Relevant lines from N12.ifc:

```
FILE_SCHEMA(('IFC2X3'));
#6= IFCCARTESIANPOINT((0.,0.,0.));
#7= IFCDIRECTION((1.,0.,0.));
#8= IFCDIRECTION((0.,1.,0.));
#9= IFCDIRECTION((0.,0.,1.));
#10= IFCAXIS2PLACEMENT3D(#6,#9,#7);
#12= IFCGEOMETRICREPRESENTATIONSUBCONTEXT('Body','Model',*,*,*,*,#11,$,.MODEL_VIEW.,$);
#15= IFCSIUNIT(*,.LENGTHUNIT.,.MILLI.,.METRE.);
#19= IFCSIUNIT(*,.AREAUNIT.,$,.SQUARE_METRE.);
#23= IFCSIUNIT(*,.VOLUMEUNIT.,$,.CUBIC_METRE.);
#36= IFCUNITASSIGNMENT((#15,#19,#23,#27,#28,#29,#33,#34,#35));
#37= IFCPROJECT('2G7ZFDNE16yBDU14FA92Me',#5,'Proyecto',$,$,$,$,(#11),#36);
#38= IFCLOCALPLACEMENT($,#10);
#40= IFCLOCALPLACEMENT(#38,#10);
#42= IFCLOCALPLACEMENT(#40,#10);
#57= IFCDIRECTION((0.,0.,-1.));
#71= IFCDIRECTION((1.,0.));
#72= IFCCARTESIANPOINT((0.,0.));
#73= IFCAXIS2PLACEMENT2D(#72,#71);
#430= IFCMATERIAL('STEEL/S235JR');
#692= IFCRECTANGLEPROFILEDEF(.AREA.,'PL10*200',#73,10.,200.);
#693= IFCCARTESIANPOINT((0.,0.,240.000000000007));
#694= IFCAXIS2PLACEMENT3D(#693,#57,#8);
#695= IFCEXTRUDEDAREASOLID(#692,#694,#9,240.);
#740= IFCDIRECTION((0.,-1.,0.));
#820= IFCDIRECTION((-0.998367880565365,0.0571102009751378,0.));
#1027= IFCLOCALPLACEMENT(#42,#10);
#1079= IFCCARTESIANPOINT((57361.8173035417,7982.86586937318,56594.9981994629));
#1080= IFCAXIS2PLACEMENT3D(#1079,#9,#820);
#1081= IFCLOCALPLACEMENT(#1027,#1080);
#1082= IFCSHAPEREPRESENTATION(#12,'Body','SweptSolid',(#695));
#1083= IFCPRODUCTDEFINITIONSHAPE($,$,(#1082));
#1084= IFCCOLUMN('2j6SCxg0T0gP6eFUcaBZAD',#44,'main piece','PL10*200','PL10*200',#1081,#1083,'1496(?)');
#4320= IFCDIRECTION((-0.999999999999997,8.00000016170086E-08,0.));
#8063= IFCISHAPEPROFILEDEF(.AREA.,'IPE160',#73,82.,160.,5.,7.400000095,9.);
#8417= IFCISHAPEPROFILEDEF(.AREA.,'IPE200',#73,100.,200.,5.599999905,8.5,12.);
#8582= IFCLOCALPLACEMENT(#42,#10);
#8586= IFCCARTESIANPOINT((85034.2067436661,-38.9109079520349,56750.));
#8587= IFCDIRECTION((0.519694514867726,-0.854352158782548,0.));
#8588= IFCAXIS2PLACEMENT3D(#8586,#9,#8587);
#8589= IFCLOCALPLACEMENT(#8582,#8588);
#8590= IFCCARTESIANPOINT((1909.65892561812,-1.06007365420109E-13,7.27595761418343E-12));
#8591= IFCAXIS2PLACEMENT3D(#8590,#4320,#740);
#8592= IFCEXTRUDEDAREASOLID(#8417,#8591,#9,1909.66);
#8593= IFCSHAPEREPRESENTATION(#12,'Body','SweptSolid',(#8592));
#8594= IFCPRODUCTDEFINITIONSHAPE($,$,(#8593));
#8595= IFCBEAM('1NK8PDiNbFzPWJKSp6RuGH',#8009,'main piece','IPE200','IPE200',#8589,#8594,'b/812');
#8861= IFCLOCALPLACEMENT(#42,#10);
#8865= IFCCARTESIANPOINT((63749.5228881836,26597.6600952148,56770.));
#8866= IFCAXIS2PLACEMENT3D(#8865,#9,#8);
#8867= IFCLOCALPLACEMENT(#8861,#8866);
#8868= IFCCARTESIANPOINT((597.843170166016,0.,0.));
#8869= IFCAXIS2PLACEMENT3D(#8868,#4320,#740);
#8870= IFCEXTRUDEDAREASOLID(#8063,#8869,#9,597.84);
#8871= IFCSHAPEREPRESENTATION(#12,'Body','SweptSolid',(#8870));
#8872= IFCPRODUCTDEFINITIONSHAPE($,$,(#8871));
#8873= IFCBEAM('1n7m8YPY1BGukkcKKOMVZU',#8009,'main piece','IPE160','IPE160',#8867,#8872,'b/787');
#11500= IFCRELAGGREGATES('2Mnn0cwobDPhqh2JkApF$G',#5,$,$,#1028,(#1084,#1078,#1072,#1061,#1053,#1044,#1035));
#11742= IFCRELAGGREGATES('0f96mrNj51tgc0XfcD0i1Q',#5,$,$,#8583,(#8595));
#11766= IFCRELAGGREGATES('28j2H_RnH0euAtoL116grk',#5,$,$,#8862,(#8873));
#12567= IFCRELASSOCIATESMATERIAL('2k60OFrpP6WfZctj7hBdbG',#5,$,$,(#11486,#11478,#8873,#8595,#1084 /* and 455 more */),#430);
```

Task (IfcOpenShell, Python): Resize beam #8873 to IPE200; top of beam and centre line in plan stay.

```python
import ifcopenshell
import ifcopenshell.util.element
import ifcopenshell.util.representation

model = ifcopenshell.open("N12.ifc")

member = model.by_guid("1n7m8YPY1BGukkcKKOMVZU")
source = next(p for p in model.by_type("IfcIShapeProfileDef") if p.ProfileName == "IPE200")

body = ifcopenshell.util.representation.get_representation(member, "Model", "Body")
solid = body.Items[0]
old_profile = solid.SweptArea

# Copy the section's sizes but keep this member's own profile position.
profile = ifcopenshell.util.element.copy(model, source)
# Profiles are centred, so shift by half the change in depth to hold the top.
shift = (old_profile.OverallDepth - profile.OverallDepth) / 2
x, y = old_profile.Position.Location.Coordinates
up = (0.0, 1.0)  # upwards, in the solid's own plane
location = model.createIfcCartesianPoint((x + up[0] * shift, y + up[1] * shift))
profile.Position = model.createIfcAxis2Placement2D(location, old_profile.Position.RefDirection)
solid.SweptArea = profile
if not model.get_total_inverses(old_profile):
    ifcopenshell.util.element.remove_deep2(model, old_profile)
member.Description = member.Description.replace("IPE160", "IPE200")
member.ObjectType = member.ObjectType.replace("IPE160", "IPE200")

print(solid.SweptArea)

model.write("N12-out.ifc")
```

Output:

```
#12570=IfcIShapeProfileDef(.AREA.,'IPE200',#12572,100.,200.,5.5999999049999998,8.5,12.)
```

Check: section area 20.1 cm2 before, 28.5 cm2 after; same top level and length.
